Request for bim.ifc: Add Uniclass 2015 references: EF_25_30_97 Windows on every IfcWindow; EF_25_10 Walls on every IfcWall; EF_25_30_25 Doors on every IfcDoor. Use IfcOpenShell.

First a look at what the model holds.

```python
import ifcopenshell

model = ifcopenshell.open("bim.ifc")
print(model.schema)
print("classifications:", [c.Name for c in model.by_type("IfcClassification")])
for ifc_class in ("IfcDoor", "IfcRoof", "IfcStair", "IfcWall", "IfcWindow"):
    print(ifc_class, len(model.by_type(ifc_class)))
```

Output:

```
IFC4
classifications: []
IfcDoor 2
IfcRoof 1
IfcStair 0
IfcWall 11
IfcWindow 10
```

```python
import ifcopenshell
import ifcopenshell.api.classification

model = ifcopenshell.open("bim.ifc")

system = ifcopenshell.api.classification.add_classification(model, classification="Uniclass 2015")

codes = {
    "IfcWindow": ("EF_25_30_97", "Windows"),
    "IfcWall": ("EF_25_10", "Walls"),
    "IfcDoor": ("EF_25_30_25", "Doors"),
}
for ifc_class, (code, name) in codes.items():
    products = model.by_type(ifc_class)
    ifcopenshell.api.classification.add_reference(
        model, products=products, classification=system, identification=code, name=name
    )
    print(code, len(products))

model.write("bim_updated.ifc")
```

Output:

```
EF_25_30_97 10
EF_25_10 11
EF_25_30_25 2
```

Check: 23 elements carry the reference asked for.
